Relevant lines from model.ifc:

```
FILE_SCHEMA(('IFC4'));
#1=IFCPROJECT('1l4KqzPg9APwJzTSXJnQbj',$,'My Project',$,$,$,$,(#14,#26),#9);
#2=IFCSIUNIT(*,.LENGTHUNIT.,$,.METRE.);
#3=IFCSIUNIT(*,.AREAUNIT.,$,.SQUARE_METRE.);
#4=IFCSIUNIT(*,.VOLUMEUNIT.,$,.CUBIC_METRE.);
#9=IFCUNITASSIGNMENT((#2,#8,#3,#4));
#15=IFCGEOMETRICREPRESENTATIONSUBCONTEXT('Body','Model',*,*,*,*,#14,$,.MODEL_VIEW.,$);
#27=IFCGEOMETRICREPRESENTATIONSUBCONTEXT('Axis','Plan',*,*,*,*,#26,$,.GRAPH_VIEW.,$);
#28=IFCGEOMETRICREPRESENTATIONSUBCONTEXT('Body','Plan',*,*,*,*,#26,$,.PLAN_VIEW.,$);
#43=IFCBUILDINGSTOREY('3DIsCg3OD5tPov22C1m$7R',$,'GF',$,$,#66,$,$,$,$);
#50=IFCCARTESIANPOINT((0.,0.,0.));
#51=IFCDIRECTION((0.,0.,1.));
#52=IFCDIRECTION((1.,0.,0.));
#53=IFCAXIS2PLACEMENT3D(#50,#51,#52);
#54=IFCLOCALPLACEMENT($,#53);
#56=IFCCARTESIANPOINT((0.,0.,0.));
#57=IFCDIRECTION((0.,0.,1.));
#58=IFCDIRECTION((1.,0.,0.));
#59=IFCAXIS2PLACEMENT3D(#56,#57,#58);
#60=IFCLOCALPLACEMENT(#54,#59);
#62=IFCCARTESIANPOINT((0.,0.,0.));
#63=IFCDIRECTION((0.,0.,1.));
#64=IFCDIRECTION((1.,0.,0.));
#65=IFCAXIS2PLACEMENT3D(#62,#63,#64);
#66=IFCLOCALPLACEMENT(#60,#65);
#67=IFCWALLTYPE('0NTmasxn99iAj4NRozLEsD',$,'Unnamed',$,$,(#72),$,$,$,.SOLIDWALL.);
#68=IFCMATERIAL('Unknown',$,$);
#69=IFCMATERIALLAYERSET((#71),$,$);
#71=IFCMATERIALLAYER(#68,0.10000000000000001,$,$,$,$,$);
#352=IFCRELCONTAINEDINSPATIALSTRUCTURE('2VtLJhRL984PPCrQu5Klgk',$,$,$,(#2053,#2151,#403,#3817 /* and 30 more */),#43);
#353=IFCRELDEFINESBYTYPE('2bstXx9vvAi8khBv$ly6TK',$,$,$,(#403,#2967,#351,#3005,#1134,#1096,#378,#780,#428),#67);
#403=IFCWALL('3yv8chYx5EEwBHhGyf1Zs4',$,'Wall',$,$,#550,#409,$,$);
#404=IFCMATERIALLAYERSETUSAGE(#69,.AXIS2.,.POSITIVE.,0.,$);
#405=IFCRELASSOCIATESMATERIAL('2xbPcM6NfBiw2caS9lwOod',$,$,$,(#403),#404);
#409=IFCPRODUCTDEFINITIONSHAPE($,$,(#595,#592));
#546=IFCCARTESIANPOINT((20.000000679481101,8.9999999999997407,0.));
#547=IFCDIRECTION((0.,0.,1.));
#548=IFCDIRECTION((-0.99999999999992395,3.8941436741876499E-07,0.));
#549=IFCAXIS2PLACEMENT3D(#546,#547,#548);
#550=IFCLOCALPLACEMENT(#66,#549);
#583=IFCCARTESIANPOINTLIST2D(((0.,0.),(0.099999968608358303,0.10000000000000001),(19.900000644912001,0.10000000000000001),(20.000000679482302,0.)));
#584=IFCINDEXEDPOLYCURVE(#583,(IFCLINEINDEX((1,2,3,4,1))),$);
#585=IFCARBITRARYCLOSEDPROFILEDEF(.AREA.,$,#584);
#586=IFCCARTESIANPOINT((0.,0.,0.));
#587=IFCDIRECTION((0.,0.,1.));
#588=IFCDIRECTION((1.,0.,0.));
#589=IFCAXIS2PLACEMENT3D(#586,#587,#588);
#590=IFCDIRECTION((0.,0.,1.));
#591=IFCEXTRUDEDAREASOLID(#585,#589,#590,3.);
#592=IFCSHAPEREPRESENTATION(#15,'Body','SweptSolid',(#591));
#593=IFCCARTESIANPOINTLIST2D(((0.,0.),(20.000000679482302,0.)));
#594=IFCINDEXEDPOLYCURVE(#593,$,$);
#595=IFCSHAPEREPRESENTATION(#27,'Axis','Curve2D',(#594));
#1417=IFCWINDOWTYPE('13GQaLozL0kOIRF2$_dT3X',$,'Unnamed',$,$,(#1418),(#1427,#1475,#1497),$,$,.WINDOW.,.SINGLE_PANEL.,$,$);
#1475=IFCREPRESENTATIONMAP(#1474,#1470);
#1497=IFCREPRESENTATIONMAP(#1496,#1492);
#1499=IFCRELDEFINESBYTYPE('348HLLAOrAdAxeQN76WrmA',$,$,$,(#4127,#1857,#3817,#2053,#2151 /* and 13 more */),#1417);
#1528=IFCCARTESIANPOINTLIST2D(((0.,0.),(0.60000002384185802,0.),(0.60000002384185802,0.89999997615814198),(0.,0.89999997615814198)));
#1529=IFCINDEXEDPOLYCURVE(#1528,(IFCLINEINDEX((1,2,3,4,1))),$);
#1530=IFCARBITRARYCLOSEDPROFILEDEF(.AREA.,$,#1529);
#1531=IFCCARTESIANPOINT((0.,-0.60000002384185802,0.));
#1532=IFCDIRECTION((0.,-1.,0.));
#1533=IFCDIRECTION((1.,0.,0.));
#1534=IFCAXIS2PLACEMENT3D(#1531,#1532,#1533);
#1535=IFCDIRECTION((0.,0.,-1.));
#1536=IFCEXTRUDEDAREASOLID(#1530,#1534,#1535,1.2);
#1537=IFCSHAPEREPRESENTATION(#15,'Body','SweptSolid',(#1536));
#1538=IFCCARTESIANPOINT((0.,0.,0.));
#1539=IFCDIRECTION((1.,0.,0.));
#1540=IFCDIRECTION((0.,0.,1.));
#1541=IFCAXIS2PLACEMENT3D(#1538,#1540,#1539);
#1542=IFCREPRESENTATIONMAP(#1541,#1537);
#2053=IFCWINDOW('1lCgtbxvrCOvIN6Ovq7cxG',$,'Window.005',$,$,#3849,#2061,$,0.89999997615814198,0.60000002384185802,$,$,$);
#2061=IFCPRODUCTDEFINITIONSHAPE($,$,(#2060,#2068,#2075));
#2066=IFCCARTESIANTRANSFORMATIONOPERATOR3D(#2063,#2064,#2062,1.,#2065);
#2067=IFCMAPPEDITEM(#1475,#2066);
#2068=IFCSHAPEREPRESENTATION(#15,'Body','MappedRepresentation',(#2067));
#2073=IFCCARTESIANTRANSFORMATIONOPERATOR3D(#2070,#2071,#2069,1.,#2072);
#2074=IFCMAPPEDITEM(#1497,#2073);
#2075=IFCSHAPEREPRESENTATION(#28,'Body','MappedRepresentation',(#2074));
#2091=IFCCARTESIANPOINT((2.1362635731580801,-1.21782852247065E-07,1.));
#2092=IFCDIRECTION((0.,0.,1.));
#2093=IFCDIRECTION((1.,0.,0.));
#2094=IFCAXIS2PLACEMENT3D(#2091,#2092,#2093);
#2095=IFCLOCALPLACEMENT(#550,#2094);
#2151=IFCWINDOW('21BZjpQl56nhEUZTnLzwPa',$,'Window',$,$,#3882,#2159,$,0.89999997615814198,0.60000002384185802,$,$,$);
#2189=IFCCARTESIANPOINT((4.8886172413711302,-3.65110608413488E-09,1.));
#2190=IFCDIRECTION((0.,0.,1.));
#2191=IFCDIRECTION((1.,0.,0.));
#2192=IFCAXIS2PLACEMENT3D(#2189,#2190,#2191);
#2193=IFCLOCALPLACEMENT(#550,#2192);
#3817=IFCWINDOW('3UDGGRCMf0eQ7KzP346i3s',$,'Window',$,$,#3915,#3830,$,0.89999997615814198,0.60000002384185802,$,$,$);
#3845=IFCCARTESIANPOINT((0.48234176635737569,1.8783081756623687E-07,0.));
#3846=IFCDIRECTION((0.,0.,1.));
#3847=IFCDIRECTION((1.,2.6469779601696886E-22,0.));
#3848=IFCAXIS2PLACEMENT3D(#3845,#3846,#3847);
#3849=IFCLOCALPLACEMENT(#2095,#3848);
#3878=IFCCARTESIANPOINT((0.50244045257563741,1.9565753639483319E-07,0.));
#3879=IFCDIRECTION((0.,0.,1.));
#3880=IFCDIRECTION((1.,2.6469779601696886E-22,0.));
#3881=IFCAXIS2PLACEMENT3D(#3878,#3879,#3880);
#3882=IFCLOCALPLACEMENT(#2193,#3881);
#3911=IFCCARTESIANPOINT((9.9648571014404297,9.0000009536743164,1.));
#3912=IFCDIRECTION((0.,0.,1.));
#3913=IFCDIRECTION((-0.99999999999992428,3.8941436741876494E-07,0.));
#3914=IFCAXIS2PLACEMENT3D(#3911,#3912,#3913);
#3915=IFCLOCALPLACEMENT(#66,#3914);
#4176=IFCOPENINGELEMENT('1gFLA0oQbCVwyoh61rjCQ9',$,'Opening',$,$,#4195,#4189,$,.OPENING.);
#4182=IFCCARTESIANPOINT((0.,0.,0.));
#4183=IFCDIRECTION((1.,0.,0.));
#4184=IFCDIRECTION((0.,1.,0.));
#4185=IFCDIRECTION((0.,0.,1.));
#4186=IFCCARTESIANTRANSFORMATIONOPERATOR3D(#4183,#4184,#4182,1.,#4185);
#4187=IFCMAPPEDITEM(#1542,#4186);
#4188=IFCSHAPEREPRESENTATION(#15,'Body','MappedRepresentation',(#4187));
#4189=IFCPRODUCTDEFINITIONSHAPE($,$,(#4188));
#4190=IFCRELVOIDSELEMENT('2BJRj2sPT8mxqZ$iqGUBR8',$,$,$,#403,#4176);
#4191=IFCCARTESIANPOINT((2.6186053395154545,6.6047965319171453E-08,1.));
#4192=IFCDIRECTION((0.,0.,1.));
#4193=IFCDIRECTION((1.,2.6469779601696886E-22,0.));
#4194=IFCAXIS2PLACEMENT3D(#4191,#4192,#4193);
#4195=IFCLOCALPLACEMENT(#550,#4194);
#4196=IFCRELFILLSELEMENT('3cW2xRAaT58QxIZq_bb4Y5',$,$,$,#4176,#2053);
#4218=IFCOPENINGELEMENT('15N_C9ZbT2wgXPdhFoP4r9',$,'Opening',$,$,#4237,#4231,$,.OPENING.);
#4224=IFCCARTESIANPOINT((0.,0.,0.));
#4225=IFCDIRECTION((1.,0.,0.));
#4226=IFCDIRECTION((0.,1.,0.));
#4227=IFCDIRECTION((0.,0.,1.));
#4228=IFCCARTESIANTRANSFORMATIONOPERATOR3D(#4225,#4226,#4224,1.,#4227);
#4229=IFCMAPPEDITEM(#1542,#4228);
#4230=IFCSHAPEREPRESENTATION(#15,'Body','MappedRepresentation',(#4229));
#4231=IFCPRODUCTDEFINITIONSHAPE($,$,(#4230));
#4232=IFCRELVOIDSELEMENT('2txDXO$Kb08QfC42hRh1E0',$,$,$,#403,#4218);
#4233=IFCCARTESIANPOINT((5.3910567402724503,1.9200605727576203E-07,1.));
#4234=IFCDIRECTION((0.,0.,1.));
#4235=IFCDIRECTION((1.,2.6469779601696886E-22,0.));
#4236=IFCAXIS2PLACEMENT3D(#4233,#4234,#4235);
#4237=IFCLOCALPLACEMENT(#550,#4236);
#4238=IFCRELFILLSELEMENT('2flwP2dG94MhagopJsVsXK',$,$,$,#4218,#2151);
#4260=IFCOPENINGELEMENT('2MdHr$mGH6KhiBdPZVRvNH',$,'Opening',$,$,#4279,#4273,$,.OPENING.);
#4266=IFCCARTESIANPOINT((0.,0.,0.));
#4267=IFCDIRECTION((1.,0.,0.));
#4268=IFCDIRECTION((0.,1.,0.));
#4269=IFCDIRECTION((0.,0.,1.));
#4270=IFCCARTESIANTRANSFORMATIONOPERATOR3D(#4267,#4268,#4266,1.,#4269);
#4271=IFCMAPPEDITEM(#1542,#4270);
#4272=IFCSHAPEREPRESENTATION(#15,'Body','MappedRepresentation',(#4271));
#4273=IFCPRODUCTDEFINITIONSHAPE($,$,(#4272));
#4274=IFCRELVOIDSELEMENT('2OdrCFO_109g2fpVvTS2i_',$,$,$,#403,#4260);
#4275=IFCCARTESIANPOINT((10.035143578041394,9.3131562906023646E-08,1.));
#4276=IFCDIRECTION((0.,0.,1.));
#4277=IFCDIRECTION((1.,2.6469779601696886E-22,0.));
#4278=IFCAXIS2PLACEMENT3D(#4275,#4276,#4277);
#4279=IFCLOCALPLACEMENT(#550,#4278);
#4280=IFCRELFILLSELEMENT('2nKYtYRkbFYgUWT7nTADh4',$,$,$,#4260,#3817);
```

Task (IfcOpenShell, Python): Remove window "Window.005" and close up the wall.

```python
import ifcopenshell
import ifcopenshell.api.feature
import ifcopenshell.api.root
import ifcopenshell.geom
import ifcopenshell.util.shape

model = ifcopenshell.open("model.ifc")
settings = ifcopenshell.geom.settings()


def volume(element):
    """Net volume in cubic metres, openings subtracted."""
    shape = ifcopenshell.geom.create_shape(settings, element)
    return ifcopenshell.util.shape.get_volume(shape.geometry)


window = model.by_guid("1lCgtbxvrCOvIN6Ovq7cxG")
opening = window.FillsVoids[0].RelatingOpeningElement
wall = opening.VoidsElements[0].RelatingBuildingElement
before = volume(wall)

ifcopenshell.api.root.remove_product(model, product=window)
ifcopenshell.api.feature.remove_feature(model, feature=opening)

after = volume(wall)

print(f"wall volume {before:.3f} -> {after:.3f} m3")

model.write("model_v2.ifc")
```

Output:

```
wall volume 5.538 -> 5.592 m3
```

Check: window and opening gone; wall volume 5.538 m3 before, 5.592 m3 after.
